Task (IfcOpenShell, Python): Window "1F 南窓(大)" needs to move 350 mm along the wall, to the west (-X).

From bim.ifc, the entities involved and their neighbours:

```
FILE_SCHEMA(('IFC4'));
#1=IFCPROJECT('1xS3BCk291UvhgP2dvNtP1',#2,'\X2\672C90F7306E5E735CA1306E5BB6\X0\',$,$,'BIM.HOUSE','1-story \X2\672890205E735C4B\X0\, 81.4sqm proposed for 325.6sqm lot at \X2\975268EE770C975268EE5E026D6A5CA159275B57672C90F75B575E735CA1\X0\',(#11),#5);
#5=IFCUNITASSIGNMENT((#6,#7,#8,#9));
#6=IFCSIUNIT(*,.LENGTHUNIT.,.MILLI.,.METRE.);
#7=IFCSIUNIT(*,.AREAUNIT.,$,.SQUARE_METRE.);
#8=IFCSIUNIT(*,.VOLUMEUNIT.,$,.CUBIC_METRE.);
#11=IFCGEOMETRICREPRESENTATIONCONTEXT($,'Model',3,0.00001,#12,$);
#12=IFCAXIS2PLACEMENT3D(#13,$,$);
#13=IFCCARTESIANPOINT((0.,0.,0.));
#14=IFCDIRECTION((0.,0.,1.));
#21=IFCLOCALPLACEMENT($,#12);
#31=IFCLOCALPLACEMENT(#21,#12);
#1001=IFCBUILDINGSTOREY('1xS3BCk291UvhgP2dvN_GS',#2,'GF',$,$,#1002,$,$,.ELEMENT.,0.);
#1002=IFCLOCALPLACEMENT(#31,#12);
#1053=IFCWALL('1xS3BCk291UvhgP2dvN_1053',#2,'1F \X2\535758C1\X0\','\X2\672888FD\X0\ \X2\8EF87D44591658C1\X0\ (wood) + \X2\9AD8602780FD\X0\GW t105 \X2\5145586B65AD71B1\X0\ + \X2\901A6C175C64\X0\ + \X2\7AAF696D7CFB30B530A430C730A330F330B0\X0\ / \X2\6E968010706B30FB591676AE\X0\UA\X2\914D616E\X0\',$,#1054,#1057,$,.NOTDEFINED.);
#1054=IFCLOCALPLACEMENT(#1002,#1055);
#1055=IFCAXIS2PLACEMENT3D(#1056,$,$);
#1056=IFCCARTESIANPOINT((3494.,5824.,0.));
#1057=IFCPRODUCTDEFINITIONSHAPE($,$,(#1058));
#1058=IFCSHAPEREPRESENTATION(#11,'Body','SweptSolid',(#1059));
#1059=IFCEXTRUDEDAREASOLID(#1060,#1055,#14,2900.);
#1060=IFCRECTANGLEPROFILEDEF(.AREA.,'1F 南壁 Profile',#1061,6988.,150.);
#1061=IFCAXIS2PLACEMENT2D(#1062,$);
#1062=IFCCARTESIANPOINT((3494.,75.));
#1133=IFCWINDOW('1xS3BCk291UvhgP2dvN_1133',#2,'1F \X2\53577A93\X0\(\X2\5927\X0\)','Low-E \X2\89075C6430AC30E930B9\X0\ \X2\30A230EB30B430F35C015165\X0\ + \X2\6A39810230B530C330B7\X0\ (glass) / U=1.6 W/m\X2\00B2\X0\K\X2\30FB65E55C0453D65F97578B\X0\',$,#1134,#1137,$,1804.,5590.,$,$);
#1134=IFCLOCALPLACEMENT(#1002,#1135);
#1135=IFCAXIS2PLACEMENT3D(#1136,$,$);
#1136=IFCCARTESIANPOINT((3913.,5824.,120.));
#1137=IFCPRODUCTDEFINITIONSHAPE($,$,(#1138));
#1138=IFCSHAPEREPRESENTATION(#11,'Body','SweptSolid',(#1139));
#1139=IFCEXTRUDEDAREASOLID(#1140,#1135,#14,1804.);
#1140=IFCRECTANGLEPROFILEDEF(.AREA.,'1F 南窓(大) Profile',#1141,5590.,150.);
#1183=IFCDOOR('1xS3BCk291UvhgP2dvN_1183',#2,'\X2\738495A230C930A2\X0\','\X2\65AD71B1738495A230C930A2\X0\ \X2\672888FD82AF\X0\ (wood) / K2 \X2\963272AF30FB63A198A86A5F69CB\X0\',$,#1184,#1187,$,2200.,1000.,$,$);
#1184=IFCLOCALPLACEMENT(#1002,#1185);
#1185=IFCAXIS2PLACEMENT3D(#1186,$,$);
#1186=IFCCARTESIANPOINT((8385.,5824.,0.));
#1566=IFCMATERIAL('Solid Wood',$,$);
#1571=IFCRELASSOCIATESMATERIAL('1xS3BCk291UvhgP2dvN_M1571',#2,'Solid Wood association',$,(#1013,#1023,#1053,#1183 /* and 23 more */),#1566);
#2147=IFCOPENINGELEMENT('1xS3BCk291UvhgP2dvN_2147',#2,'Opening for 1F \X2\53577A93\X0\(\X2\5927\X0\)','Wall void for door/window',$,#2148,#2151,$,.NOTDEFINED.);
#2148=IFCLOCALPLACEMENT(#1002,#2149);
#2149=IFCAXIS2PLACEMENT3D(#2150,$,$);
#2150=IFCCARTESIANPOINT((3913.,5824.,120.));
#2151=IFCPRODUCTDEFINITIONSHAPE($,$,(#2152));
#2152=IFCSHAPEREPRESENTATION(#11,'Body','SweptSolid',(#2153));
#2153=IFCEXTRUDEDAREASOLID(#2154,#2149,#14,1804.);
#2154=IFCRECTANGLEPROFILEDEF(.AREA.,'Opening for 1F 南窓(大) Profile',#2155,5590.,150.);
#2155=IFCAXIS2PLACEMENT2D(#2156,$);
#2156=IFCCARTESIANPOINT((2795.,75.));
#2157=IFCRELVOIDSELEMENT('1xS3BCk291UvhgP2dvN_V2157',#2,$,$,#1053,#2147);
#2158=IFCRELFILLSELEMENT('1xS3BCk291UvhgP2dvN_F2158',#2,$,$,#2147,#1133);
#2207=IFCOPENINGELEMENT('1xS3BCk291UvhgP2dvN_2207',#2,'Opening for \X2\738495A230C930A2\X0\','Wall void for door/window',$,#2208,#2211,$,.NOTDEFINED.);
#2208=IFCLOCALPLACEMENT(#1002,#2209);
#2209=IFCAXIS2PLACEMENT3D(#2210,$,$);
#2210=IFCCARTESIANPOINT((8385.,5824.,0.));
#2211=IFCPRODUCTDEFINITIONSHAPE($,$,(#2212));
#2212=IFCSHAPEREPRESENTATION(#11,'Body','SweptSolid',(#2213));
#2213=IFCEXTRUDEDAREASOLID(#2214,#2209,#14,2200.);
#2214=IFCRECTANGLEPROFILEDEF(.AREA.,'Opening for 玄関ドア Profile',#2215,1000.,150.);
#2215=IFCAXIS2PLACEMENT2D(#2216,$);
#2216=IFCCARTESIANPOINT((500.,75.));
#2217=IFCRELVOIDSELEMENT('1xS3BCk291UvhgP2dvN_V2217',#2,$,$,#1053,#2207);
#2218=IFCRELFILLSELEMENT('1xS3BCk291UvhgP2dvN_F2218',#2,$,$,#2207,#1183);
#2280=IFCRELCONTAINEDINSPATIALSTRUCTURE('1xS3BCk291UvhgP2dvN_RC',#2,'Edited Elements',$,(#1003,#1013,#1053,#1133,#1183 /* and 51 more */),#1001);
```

```python
import ifcopenshell
import ifcopenshell.api.geometry
import ifcopenshell.util.placement

model = ifcopenshell.open("bim.ifc")

window = model.by_guid("1xS3BCk291UvhgP2dvN_1133")
opening = window.FillsVoids[0].RelatingOpeningElement
wall = opening.VoidsElements[0].RelatingBuildingElement

wall_matrix = ifcopenshell.util.placement.get_local_placement(wall.ObjectPlacement)
shift = wall_matrix[:3, 0] * -350.0
before = ifcopenshell.util.placement.get_local_placement(window.ObjectPlacement)[:3, 3].copy()

# The window is not placed relative to its opening, so move both.
for product in (opening, window):
    matrix = ifcopenshell.util.placement.get_local_placement(product.ObjectPlacement)
    matrix[:3, 3] += shift
    ifcopenshell.api.geometry.edit_object_placement(model, product=product, matrix=matrix, is_si=False)

after = ifcopenshell.util.placement.get_local_placement(window.ObjectPlacement)[:3, 3]
print("window moved by", (after - before).round(3) + 0.0)

model.write("bim_v2.ifc")
```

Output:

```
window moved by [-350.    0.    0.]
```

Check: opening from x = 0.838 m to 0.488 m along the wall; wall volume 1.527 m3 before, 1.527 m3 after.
